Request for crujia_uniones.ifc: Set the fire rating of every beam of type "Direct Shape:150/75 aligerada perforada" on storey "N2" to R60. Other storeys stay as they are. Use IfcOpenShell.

First a look at what the model holds.

```python
import ifcopenshell
import ifcopenshell.util.element

model = ifcopenshell.open("crujia_uniones.ifc")
print(model.schema)
storey = next(s for s in model.by_type("IfcBuildingStorey") if s.Name == "N2")
beams = [e for e in ifcopenshell.util.element.get_decomposition(storey) if e.is_a("IfcBeam")]
seen = {}
for e in beams:
    element_type = ifcopenshell.util.element.get_type(e)
    key = (element_type.Name if element_type != e and element_type else None, ifcopenshell.util.element.get_pset(e, "Pset_BeamCommon", "FireRating"))
    seen[key] = seen.get(key, 0) + 1
for (name, value), count in sorted(seen.items(), key=str):
    print(count, "x", name, "|", value)
```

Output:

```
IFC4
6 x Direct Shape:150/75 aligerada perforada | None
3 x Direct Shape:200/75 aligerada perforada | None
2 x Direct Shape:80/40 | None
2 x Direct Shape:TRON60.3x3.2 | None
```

```python
import ifcopenshell
import ifcopenshell.api.pset
import ifcopenshell.util.element

model = ifcopenshell.open("crujia_uniones.ifc")

storey = next(s for s in model.by_type("IfcBuildingStorey") if s.Name == "N2")
beams = [e for e in ifcopenshell.util.element.get_decomposition(storey) if e.is_a("IfcBeam")]

count = 0
for e in beams:
    element_type = ifcopenshell.util.element.get_type(e)
    if element_type in (None, e) or element_type.Name != "Direct Shape:150/75 aligerada perforada":
        continue
    # add_pset returns the element's existing set when there is one.
    pset = ifcopenshell.api.pset.add_pset(model, product=e, name="Pset_BeamCommon")
    ifcopenshell.api.pset.edit_pset(model, pset=pset, properties={"FireRating": "R60"})
    count += 1

print(count, "beams updated")

model.write("crujia_uniones-out.ifc")
```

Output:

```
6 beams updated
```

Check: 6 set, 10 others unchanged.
